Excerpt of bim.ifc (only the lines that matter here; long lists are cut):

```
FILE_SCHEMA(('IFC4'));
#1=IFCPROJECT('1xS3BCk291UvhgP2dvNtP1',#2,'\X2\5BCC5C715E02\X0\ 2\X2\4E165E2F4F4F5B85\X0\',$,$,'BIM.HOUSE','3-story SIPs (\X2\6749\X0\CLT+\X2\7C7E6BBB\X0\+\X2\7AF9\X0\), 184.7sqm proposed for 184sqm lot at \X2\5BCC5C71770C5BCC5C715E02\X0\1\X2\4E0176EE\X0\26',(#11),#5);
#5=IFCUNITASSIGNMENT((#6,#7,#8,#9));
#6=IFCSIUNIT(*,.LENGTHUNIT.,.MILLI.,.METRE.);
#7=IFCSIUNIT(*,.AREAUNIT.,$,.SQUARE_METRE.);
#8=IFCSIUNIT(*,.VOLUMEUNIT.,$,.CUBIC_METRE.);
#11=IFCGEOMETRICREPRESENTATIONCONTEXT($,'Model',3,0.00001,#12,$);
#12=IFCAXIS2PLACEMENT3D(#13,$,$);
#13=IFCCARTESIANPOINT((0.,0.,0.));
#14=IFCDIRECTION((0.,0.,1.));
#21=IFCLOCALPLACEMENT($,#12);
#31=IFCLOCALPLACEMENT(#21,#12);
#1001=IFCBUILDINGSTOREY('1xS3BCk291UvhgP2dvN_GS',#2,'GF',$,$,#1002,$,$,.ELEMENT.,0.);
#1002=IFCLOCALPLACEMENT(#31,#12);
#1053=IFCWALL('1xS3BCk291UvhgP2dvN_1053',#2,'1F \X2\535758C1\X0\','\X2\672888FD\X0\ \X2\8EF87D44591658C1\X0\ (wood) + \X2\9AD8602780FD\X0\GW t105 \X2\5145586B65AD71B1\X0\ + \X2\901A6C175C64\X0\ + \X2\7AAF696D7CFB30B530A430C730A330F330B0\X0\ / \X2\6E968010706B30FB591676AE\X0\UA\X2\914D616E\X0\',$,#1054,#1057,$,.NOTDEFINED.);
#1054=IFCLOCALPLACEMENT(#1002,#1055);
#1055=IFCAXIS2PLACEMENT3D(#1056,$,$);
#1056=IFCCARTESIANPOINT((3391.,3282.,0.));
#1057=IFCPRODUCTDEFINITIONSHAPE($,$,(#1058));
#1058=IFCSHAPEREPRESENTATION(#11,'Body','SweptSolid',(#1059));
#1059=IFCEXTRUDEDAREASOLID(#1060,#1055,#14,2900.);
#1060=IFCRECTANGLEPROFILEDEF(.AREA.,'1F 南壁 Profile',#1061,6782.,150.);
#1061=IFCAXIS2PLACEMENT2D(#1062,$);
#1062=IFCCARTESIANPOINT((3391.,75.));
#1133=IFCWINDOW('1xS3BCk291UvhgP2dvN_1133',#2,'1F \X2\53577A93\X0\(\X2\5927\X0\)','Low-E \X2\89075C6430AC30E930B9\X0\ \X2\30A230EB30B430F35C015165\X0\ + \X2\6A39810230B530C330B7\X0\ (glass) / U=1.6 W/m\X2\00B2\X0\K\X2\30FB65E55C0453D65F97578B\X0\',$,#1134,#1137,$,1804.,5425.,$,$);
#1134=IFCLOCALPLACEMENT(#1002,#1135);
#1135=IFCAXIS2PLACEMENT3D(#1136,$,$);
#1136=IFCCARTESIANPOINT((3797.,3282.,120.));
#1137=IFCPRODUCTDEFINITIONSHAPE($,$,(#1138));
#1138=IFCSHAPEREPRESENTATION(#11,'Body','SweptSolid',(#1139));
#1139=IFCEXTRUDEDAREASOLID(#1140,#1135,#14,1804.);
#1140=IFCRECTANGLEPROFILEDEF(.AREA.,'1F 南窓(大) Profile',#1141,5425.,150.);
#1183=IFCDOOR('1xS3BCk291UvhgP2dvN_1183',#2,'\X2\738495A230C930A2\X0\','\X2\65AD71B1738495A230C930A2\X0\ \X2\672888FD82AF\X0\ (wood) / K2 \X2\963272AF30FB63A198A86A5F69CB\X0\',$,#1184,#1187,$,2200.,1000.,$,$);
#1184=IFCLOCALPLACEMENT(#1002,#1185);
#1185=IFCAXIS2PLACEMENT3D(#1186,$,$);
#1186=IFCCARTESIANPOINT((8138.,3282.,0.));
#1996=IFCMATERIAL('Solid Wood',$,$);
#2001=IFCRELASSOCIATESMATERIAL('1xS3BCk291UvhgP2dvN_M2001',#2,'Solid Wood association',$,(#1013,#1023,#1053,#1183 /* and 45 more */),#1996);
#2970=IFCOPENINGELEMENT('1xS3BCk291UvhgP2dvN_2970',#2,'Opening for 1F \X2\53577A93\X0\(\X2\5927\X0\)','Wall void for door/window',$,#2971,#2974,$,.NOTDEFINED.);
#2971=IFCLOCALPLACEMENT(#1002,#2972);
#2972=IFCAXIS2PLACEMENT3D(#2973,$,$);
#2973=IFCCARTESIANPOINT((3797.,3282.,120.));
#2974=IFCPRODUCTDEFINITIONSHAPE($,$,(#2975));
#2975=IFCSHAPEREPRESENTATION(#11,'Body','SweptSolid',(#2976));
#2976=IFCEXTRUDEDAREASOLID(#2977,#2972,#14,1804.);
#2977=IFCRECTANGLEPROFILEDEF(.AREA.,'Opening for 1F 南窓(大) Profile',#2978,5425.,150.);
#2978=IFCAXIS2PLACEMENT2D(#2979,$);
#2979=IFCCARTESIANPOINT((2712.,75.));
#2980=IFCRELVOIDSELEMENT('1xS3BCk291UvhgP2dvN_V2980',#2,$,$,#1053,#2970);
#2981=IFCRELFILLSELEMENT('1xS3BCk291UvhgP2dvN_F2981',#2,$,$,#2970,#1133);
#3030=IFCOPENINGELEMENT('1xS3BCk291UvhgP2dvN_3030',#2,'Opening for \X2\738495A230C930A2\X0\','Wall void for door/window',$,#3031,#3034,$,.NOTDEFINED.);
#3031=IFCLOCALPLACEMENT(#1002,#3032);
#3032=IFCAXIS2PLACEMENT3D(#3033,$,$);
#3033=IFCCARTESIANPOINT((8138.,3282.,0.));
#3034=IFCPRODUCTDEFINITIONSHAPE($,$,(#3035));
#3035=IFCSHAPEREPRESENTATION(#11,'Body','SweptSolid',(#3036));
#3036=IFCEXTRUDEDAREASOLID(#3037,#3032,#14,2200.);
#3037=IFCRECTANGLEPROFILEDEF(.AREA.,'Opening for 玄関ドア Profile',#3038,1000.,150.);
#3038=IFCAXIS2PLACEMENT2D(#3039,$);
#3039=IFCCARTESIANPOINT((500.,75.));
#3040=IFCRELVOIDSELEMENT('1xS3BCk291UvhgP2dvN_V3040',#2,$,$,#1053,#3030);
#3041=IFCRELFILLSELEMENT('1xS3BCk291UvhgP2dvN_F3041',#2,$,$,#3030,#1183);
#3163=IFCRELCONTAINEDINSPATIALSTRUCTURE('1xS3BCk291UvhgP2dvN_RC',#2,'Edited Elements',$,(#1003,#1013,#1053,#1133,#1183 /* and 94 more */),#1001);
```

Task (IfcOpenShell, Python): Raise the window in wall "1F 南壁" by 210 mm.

```python
import numpy as np
import ifcopenshell
import ifcopenshell.api.geometry
import ifcopenshell.util.placement
import ifcopenshell.util.unit

model = ifcopenshell.open("bim.ifc")
unit_scale = ifcopenshell.util.unit.calculate_unit_scale(model)

window = model.by_guid("1xS3BCk291UvhgP2dvN_1133")
opening = window.FillsVoids[0].RelatingOpeningElement
dz = 0.21 / unit_scale

shift = np.array([0.0, 0.0, dz])
# The window is not placed relative to its opening, so move both.
for product in (opening, window):
    matrix = ifcopenshell.util.placement.get_local_placement(product.ObjectPlacement)
    matrix[:3, 3] += shift
    ifcopenshell.api.geometry.edit_object_placement(model, product=product, matrix=matrix, is_si=False)

print(f"moved by {dz * unit_scale:+.3f} m")

model.write("bim_rev.ifc")
```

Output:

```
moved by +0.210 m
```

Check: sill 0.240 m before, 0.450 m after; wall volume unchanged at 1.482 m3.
